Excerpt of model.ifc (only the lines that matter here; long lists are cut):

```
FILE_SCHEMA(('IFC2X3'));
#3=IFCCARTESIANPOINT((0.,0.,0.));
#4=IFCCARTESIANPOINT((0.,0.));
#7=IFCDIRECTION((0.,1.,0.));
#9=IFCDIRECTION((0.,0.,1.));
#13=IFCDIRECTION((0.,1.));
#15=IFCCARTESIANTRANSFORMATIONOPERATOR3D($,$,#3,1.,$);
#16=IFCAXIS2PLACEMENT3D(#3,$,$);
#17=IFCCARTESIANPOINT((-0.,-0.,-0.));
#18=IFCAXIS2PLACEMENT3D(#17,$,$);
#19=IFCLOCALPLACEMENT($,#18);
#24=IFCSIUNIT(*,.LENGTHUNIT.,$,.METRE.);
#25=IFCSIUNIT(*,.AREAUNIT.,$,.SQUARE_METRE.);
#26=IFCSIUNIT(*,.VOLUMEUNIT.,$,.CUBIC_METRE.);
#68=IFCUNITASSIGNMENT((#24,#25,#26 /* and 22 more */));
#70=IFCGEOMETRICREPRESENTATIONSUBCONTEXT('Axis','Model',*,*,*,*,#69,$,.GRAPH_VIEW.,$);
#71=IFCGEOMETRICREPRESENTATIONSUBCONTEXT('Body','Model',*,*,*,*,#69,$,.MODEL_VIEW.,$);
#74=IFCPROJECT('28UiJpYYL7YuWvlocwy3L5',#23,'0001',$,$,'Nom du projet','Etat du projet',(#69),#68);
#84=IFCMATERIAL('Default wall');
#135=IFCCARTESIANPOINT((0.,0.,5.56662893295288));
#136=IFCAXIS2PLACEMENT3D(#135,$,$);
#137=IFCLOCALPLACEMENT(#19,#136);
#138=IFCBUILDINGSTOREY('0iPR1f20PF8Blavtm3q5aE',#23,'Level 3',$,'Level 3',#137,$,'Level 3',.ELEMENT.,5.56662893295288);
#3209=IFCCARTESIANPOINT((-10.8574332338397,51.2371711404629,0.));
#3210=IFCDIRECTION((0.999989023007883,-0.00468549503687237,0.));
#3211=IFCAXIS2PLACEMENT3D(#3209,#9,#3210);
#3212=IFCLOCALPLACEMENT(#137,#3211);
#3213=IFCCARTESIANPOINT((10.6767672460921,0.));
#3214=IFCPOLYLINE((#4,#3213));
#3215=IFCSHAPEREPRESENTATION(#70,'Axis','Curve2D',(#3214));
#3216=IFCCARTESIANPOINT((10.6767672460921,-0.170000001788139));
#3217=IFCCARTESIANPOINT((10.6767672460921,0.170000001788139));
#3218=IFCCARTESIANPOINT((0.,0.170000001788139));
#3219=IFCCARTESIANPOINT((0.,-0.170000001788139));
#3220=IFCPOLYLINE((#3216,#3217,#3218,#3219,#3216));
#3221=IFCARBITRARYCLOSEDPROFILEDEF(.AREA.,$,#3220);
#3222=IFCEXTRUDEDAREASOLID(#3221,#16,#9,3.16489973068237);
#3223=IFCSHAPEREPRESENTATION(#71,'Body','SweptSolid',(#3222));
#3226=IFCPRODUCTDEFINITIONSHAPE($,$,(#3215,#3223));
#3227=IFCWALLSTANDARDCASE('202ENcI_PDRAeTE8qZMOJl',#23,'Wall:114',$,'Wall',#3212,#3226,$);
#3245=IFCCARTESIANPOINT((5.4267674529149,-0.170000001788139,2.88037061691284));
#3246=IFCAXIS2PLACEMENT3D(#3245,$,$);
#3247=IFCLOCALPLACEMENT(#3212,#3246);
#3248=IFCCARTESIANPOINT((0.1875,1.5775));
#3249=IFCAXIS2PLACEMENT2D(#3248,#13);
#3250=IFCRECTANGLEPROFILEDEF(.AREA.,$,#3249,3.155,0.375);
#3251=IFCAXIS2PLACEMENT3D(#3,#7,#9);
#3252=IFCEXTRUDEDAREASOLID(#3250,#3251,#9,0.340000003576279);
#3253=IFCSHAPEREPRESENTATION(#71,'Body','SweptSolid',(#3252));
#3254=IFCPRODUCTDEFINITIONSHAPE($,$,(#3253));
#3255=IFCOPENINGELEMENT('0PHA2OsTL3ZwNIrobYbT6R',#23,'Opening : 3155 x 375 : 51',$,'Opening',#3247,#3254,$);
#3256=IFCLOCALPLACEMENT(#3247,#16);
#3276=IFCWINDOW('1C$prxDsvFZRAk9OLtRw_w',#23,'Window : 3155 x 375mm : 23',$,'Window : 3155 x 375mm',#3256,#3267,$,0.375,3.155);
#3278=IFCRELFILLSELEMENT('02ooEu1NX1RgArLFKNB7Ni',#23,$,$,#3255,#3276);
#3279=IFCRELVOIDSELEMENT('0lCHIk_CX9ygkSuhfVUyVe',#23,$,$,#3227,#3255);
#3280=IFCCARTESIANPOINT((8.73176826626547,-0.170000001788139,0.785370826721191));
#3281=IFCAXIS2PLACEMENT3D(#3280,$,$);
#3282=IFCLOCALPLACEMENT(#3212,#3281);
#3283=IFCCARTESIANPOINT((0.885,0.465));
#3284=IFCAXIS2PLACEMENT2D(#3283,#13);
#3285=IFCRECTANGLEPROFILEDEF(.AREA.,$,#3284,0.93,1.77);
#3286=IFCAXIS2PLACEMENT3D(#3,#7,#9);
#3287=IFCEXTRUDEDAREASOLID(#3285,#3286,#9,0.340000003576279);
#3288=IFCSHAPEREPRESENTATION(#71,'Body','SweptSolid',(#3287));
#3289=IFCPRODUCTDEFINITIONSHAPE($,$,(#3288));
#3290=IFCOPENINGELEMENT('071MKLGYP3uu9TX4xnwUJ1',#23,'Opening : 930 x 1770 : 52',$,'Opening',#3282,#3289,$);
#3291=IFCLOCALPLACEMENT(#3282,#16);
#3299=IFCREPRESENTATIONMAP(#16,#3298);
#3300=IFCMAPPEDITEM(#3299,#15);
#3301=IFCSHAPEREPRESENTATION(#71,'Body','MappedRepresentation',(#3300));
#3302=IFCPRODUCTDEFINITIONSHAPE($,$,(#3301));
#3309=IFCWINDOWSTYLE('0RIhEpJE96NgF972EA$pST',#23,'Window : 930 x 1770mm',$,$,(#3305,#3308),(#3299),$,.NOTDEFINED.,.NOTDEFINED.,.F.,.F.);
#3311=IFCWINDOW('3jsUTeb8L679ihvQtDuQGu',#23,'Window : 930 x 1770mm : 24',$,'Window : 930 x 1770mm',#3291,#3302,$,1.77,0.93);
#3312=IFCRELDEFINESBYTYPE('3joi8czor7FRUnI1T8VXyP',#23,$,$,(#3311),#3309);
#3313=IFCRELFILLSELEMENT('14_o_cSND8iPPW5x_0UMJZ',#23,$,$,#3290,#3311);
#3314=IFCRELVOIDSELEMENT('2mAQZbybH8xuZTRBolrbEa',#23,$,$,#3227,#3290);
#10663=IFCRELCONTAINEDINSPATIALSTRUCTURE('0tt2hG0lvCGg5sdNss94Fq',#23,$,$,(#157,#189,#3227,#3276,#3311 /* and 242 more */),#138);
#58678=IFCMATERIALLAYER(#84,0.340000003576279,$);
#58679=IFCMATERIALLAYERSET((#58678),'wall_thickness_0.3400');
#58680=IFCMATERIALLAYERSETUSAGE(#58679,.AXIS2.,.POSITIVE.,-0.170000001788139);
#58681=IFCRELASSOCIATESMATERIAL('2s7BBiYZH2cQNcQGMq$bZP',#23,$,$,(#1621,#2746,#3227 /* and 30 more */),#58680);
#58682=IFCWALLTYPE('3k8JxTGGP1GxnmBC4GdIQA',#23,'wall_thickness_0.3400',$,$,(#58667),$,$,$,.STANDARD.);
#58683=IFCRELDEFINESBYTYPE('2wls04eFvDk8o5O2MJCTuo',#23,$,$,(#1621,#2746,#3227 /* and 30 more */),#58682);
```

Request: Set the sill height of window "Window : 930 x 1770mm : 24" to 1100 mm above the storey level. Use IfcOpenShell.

```python
import numpy as np
import ifcopenshell
import ifcopenshell.api.geometry
import ifcopenshell.geom
import ifcopenshell.util.element
import ifcopenshell.util.placement
import ifcopenshell.util.shape
import ifcopenshell.util.unit

model = ifcopenshell.open("model.ifc")
unit_scale = ifcopenshell.util.unit.calculate_unit_scale(model)

window = model.by_guid("3jsUTeb8L679ihvQtDuQGu")
opening = window.FillsVoids[0].RelatingOpeningElement
storey = ifcopenshell.util.element.get_container(window, ifc_class="IfcBuildingStorey")
level = ifcopenshell.util.placement.get_local_placement(storey.ObjectPlacement)[2, 3]

# The opening's origin need not be at the sill, so measure its lowest point.
shape = ifcopenshell.geom.create_shape(ifcopenshell.geom.settings(), opening)
bottom = ifcopenshell.util.shape.get_shape_bottom_elevation(shape, shape.geometry) / unit_scale
dz = level + 1.1 - bottom

shift = np.array([0.0, 0.0, dz])
# The window is placed relative to its opening, so it follows when the opening moves.
matrix = ifcopenshell.util.placement.get_local_placement(opening.ObjectPlacement)
matrix[:3, 3] += shift
ifcopenshell.api.geometry.edit_object_placement(
    model, product=opening, matrix=matrix, is_si=False, should_transform_children=True
)

print(f"moved by {dz * unit_scale:+.3f} m")

model.write("model_updated.ifc")
```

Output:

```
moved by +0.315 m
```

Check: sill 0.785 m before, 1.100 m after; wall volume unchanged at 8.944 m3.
